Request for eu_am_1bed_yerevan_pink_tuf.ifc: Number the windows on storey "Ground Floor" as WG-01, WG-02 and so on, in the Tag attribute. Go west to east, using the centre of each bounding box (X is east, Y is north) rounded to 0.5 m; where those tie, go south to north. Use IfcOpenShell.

First a look at what the model holds.

```python
import ifcopenshell
import ifcopenshell.util.element
import ifcopenshell.util.placement

model = ifcopenshell.open("eu_am_1bed_yerevan_pink_tuf.ifc")
print(model.schema)
storey = next(s for s in model.by_type("IfcBuildingStorey") if s.Name == "Ground Floor")
windows = [e for e in ifcopenshell.util.element.get_decomposition(storey) if e.is_a("IfcWindow")]
for e in sorted(windows, key=lambda e: e.id()):
    origin = ifcopenshell.util.placement.get_local_placement(e.ObjectPlacement)[:3, 3]
    print(e.id(), e.Tag, e.Name, origin.round(2) + 0.0, sep=" | ")
```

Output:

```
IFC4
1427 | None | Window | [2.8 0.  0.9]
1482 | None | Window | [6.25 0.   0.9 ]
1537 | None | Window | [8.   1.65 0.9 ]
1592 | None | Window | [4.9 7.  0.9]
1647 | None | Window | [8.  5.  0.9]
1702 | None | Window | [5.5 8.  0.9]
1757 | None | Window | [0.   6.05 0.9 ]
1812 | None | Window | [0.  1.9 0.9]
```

```python
import ifcopenshell
import ifcopenshell.geom
import ifcopenshell.util.element
import ifcopenshell.util.shape

model = ifcopenshell.open("eu_am_1bed_yerevan_pink_tuf.ifc")
settings = ifcopenshell.geom.settings()
settings.set("use-world-coords", True)


def centre(element):
    shape = ifcopenshell.geom.create_shape(settings, element)
    return ifcopenshell.util.shape.get_bbox_centroid(shape.geometry)


storey = next(s for s in model.by_type("IfcBuildingStorey") if s.Name == "Ground Floor")
windows = [e for e in ifcopenshell.util.element.get_decomposition(storey) if e.is_a("IfcWindow")]

# Insertion points can sit at a corner or the storey origin, so sort by the geometry (in metres).
centres = {e: centre(e) for e in windows}
windows.sort(key=lambda e: (round(centres[e][0] / 0.5), centres[e][1]))

for i, e in enumerate(windows, start=1):
    number = f"WG-{i:02d}"
    e.Tag = number
    print(e.id(), number)

model.write("eu_am_1bed_yerevan_pink_tuf_updated.ifc")
```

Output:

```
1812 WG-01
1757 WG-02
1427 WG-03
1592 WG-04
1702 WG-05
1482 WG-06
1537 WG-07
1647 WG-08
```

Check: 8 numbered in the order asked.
